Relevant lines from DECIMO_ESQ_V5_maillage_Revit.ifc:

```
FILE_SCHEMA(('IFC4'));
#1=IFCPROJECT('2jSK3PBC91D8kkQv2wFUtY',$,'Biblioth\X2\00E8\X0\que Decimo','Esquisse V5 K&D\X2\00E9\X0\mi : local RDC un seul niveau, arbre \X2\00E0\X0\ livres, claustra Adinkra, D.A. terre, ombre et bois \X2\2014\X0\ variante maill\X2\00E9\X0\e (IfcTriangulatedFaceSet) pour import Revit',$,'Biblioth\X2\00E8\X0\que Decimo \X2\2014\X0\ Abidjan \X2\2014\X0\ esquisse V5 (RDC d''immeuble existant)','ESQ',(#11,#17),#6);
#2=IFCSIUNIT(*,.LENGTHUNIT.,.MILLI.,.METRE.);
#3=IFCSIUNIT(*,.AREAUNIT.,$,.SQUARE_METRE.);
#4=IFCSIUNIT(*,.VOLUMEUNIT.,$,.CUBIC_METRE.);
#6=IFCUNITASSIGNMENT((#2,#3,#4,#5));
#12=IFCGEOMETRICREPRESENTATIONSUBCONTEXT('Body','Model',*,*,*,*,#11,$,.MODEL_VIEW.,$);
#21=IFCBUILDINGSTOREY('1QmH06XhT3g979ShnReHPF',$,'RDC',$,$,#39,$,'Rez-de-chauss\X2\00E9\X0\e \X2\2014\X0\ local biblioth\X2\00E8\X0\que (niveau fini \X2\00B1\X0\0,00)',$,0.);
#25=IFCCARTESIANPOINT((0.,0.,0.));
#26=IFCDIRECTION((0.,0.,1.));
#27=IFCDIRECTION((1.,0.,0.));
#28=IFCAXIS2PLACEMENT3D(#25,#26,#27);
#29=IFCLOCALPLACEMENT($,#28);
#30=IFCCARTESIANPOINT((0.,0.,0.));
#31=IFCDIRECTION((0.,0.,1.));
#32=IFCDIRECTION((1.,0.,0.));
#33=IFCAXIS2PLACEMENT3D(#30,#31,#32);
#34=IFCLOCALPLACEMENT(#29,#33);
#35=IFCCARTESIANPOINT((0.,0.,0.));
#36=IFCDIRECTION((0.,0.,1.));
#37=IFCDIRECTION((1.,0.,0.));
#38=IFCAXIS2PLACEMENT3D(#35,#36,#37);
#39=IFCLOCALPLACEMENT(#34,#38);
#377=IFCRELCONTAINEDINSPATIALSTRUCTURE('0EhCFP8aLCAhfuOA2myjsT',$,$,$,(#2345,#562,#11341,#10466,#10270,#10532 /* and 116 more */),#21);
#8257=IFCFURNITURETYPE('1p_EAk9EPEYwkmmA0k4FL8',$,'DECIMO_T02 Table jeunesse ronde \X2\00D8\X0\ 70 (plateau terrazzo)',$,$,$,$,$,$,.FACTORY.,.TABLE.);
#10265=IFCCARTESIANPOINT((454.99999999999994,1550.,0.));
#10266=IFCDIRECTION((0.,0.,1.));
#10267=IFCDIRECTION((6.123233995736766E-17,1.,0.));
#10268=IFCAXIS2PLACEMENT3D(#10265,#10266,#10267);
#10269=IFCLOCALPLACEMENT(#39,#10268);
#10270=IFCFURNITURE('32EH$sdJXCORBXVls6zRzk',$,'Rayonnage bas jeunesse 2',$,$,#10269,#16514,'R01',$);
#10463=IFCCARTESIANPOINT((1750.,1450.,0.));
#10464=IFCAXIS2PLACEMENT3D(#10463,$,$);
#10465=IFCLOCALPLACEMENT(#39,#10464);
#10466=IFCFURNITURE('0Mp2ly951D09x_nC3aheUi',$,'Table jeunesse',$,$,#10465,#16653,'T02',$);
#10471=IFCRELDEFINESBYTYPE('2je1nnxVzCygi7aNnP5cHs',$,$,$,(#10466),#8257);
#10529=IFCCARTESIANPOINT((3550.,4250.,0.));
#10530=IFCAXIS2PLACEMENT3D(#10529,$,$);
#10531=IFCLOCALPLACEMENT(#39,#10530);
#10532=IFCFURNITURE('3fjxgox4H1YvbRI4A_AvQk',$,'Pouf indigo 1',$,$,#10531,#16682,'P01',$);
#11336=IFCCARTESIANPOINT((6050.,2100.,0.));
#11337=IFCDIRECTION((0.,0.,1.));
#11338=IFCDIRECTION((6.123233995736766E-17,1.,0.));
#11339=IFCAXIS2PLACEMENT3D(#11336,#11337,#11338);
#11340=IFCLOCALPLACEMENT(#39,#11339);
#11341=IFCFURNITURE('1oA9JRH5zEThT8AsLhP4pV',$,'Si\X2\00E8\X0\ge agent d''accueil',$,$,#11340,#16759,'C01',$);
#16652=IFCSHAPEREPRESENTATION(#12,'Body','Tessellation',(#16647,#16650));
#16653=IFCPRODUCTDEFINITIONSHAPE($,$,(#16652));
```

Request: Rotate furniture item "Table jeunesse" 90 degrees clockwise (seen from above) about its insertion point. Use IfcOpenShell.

```python
import ifcopenshell
import ifcopenshell.api.geometry
import ifcopenshell.util.placement

model = ifcopenshell.open("DECIMO_ESQ_V5_maillage_Revit.ifc")

item = model.by_guid("0Mp2ly951D09x_nC3aheUi")
matrix = ifcopenshell.util.placement.get_local_placement(item.ObjectPlacement)
matrix = matrix @ ifcopenshell.util.placement.rotation(-90, "Z")
ifcopenshell.api.geometry.edit_object_placement(model, product=item, matrix=matrix, is_si=False)

print(ifcopenshell.util.placement.get_local_placement(item.ObjectPlacement).round(3) + 0.0)

model.write("DECIMO_ESQ_V5_maillage_Revit_edited.ifc")
```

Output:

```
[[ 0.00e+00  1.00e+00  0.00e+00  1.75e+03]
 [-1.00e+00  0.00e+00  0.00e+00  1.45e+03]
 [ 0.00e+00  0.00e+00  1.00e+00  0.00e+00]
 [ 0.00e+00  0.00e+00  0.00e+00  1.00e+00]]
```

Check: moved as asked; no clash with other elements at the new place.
